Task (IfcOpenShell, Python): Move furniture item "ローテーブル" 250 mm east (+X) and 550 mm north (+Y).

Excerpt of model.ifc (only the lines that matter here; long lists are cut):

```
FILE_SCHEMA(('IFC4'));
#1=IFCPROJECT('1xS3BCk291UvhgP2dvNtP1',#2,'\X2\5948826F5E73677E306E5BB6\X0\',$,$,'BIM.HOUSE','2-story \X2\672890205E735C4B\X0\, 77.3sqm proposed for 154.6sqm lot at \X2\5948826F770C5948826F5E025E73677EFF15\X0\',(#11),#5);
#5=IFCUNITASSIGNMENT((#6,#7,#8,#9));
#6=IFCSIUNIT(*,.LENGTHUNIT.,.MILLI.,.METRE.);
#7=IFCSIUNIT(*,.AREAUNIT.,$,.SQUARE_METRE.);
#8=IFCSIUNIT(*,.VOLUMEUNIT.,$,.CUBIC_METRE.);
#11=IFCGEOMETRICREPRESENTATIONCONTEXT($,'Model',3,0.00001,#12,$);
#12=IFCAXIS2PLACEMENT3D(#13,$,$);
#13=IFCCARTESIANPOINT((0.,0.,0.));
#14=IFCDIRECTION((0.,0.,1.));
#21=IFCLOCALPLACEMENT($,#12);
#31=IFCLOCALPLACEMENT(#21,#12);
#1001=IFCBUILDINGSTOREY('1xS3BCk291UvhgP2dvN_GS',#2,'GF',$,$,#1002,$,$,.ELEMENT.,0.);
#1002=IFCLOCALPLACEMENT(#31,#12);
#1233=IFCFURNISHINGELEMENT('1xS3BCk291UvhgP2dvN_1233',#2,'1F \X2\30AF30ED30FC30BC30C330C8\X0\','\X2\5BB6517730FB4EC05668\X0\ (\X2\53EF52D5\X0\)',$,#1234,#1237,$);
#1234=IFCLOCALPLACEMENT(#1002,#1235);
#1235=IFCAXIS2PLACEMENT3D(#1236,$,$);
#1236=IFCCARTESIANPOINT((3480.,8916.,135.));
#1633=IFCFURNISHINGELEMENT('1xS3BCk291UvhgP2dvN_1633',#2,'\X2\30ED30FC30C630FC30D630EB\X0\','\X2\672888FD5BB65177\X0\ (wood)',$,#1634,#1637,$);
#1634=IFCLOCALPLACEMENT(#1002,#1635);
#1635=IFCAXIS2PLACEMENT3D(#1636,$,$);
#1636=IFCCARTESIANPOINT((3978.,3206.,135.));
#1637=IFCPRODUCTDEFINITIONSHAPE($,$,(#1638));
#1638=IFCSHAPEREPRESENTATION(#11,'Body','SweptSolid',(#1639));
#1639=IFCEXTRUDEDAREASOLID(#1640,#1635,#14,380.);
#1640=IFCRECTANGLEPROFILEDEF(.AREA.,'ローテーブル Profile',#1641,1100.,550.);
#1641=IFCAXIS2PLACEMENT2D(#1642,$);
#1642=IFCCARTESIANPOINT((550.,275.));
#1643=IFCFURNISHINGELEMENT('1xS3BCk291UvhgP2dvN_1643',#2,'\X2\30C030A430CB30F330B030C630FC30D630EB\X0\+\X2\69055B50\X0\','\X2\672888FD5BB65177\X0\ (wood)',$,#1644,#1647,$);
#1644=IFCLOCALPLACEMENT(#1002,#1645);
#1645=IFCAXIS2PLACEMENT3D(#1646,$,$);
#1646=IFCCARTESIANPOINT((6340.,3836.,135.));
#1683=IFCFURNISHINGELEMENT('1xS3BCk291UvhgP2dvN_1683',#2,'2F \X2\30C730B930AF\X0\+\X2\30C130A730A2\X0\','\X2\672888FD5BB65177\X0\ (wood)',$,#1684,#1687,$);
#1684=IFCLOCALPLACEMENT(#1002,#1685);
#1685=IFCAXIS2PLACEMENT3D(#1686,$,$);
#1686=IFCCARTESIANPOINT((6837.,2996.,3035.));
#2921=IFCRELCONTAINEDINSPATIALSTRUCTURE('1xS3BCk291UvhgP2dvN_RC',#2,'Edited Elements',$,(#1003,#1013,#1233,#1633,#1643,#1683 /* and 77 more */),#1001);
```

```python
import ifcopenshell
import ifcopenshell.api.geometry
import ifcopenshell.util.placement
import ifcopenshell.util.unit

model = ifcopenshell.open("model.ifc")
unit_scale = ifcopenshell.util.unit.calculate_unit_scale(model)

item = model.by_id(1633)
matrix = ifcopenshell.util.placement.get_local_placement(item.ObjectPlacement)
matrix[0, 3] += 0.25 / unit_scale
matrix[1, 3] += 0.55 / unit_scale
ifcopenshell.api.geometry.edit_object_placement(model, product=item, matrix=matrix, is_si=False)

print(ifcopenshell.util.placement.get_local_placement(item.ObjectPlacement).round(3) + 0.0)

model.write("model_v2.ifc")
```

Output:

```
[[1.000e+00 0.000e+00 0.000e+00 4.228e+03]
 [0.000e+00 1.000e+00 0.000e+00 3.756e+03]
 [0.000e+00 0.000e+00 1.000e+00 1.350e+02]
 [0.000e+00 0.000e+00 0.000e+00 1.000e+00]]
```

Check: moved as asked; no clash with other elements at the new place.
